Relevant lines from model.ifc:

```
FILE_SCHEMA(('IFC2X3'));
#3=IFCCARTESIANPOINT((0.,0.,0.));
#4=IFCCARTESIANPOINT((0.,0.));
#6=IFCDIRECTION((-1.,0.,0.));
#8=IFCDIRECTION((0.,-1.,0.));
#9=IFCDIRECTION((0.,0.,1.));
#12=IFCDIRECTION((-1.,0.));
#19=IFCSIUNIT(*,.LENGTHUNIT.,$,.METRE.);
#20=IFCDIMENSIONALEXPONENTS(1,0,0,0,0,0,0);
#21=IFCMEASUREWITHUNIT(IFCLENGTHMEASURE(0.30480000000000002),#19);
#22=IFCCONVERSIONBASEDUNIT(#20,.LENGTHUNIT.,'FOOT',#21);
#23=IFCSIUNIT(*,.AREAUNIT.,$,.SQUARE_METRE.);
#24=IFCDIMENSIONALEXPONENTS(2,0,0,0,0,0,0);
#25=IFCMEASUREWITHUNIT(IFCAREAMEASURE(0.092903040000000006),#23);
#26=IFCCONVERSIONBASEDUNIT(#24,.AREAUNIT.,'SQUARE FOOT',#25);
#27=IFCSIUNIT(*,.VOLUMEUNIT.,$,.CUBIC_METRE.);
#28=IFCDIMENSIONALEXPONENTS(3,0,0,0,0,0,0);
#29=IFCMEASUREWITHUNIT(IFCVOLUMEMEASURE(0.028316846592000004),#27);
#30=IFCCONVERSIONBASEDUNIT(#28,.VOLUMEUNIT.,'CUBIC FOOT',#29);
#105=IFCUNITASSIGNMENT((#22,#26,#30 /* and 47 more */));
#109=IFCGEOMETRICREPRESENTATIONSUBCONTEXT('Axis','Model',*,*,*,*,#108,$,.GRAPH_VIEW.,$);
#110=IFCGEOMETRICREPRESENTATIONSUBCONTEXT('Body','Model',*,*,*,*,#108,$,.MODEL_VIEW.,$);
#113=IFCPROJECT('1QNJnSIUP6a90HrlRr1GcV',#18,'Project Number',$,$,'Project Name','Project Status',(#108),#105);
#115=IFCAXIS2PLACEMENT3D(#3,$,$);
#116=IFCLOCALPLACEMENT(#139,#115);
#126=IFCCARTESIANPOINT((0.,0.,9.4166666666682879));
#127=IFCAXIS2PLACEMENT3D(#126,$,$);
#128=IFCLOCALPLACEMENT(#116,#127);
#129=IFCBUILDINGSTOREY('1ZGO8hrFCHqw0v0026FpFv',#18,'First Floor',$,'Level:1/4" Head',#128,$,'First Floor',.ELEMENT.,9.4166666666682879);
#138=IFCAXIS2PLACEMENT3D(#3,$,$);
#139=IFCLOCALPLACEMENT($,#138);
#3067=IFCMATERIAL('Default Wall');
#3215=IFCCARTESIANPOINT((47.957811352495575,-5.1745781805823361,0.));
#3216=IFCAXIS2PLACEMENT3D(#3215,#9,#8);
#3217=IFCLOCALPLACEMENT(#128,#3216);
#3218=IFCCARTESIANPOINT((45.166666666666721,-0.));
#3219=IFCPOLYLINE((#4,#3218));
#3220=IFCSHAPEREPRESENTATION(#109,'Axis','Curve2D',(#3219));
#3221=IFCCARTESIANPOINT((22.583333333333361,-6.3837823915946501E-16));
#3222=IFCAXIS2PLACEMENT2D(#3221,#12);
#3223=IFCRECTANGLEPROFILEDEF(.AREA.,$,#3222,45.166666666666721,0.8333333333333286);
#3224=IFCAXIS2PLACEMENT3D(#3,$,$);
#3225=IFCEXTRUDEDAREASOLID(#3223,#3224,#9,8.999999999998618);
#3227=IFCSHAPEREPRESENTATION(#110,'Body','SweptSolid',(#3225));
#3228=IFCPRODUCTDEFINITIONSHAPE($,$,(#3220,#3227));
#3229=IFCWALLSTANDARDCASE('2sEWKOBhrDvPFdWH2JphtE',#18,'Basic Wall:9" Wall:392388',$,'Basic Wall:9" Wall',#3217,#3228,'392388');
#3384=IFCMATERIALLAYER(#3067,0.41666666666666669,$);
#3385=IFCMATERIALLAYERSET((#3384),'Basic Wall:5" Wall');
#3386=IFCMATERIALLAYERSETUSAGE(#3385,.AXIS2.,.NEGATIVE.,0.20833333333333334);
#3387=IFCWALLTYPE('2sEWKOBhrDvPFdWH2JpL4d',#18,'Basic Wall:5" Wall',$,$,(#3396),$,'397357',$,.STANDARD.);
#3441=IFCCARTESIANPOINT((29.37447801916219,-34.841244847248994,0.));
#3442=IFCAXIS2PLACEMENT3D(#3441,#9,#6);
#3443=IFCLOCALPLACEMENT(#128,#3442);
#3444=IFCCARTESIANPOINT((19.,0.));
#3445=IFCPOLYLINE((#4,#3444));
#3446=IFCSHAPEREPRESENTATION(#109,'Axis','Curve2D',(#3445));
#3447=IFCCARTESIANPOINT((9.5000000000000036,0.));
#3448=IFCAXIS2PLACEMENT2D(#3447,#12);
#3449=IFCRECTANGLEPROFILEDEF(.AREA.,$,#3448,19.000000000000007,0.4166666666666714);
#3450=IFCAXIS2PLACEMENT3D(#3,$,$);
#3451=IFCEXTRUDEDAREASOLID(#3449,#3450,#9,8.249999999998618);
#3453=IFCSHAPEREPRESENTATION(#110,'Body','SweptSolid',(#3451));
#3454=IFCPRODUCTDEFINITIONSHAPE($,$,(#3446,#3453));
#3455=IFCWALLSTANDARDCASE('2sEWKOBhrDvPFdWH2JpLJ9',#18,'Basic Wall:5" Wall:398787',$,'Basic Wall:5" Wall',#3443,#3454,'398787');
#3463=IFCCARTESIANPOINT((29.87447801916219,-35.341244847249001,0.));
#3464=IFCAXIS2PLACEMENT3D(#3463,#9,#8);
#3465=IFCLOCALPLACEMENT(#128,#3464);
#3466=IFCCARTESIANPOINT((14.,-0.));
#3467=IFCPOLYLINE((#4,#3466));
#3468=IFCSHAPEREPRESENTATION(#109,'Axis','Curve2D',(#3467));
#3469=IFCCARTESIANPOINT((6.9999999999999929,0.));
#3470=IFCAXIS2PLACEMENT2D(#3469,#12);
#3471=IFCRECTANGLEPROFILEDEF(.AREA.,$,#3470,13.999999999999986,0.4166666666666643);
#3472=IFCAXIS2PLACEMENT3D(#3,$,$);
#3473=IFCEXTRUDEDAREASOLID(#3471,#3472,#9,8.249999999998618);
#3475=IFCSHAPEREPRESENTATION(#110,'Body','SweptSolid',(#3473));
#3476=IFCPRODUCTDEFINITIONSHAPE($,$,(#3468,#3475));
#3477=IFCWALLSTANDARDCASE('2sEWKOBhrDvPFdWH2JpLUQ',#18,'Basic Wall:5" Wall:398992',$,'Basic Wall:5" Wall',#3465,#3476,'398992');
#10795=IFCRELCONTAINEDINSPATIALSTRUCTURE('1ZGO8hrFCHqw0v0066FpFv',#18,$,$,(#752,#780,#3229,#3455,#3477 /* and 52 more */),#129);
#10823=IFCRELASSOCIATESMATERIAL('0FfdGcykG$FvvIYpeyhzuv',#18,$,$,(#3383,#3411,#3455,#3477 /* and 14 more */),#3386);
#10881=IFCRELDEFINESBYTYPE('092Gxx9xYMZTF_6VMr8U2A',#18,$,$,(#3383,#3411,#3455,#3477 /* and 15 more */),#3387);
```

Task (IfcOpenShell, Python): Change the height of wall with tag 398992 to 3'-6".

```python
import ifcopenshell
import ifcopenshell.geom
import ifcopenshell.util.representation
import ifcopenshell.util.shape
import ifcopenshell.util.unit

model = ifcopenshell.open("model.ifc")
unit_scale = ifcopenshell.util.unit.calculate_unit_scale(model)
settings = ifcopenshell.geom.settings()


def volume(element):
    """Net volume in cubic metres, openings subtracted."""
    shape = ifcopenshell.geom.create_shape(settings, element)
    return ifcopenshell.util.shape.get_volume(shape.geometry)


wall = model.by_id(3477)
before = volume(wall)

body = ifcopenshell.util.representation.get_representation(wall, "Model", "Body")
solid = body.Items[0]
old_height = solid.Depth
solid.Depth = 42 * 0.0254 / unit_scale
after = volume(wall)

print(f"height {old_height:g} -> {solid.Depth:g}, volume {before:.3f} -> {after:.3f} m3")

model.write("model_v2.ifc")
```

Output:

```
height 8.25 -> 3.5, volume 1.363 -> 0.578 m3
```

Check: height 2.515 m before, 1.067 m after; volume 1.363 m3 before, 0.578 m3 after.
